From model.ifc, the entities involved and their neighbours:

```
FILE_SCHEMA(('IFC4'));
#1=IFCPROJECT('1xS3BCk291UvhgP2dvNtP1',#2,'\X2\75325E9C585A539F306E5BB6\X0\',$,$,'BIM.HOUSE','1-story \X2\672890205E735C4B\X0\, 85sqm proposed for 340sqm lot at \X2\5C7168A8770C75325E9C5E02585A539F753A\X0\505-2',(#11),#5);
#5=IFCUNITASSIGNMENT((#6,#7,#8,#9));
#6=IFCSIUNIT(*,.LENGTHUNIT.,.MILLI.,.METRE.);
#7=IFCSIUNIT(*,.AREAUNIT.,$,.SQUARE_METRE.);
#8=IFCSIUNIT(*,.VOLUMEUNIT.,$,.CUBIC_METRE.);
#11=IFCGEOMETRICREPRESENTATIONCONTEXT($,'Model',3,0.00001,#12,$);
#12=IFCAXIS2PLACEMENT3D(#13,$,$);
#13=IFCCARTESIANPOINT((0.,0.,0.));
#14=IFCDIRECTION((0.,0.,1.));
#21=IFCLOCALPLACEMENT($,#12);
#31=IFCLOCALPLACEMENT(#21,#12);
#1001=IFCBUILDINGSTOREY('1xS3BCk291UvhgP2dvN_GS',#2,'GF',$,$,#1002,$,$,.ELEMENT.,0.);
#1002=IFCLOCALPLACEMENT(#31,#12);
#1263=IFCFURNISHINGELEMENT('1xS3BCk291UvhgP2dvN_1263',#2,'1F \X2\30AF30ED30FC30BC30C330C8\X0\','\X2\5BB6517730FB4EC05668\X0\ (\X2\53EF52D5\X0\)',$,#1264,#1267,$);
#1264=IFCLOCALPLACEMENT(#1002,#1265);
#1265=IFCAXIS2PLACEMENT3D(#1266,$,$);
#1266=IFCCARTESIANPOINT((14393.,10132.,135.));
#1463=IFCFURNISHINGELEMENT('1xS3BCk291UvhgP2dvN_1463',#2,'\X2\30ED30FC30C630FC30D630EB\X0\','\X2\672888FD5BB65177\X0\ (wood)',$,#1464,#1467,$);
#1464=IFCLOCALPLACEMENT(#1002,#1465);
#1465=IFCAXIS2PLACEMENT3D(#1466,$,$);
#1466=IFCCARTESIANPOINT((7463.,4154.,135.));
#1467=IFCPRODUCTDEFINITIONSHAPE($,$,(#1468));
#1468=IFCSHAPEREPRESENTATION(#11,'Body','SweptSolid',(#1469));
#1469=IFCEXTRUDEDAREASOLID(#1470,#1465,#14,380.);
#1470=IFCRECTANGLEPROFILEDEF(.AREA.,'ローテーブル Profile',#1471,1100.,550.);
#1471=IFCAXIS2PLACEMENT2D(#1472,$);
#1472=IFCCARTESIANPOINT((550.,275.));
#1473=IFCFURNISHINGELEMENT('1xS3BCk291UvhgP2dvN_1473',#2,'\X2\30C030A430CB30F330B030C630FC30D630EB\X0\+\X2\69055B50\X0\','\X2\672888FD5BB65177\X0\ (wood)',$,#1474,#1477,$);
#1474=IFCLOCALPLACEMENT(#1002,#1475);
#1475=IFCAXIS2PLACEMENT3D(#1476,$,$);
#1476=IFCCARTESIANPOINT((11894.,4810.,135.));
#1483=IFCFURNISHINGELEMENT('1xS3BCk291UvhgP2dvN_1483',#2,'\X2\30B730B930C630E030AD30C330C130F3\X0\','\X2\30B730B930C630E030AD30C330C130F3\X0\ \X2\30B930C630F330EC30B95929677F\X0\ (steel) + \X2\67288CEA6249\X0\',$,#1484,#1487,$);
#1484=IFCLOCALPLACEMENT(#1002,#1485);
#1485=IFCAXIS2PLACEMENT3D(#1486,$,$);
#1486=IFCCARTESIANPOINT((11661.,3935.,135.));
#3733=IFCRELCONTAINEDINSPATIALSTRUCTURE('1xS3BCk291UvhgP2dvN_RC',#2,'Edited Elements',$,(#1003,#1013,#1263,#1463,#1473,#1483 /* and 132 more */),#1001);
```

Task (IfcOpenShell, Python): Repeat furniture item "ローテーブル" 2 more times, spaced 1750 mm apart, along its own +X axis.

```python
import ifcopenshell
import ifcopenshell.api.geometry
import ifcopenshell.api.root
import ifcopenshell.util.element
import ifcopenshell.util.placement
import ifcopenshell.util.unit

model = ifcopenshell.open("model.ifc")
unit_scale = ifcopenshell.util.unit.calculate_unit_scale(model)


def reuse_history(source, copy):
    """copy_class also copies each property set's owner history, people and application; keep the originals."""
    for rel in copy.IsDefinedBy:
        if rel.is_a("IfcRelDefinesByProperties") and (history := rel.RelatingPropertyDefinition.OwnerHistory):
            rel.RelatingPropertyDefinition.OwnerHistory = source.OwnerHistory
            ifcopenshell.util.element.remove_deep2(model, history)


source = model.by_id(1463)
base = ifcopenshell.util.placement.get_local_placement(source.ObjectPlacement)
step = base[:3, 0] * 1.75 / unit_scale

for i in range(1, 3):
    copy = ifcopenshell.api.root.copy_class(model, product=source)
    copy.Representation = ifcopenshell.util.element.copy_deep(
        model, source.Representation, exclude=["IfcGeometricRepresentationContext", "IfcRepresentationMap"]
    )
    reuse_history(source, copy)
    matrix = base.copy()
    matrix[:3, 3] += i * step
    print("added at", matrix[:3, 3].round(3) + 0.0)
    ifcopenshell.api.geometry.edit_object_placement(model, product=copy, matrix=matrix, is_si=False)

model.write("model_edited.ifc")
```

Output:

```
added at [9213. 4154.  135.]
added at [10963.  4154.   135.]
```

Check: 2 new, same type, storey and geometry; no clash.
